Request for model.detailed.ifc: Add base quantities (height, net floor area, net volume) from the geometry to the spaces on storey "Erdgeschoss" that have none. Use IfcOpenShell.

First a look at what the model holds.

```python
import ifcopenshell
import ifcopenshell.util.element
import ifcopenshell.util.unit

model = ifcopenshell.open("model.detailed.ifc")
print(model.schema)
for unit_type in ("LENGTHUNIT", "AREAUNIT", "VOLUMEUNIT"):
    print(unit_type, ifcopenshell.util.unit.calculate_unit_scale(model, unit_type))
storey = next(s for s in model.by_type("IfcBuildingStorey") if s.Name == "Erdgeschoss")
spaces = [e for e in ifcopenshell.util.element.get_decomposition(storey) if e.is_a("IfcSpace")]
for e in sorted(spaces, key=lambda e: e.id()):
    print(e.id(), e.is_a(), e.Name, list(ifcopenshell.util.element.get_psets(e, qtos_only=True)), sep=" | ")
```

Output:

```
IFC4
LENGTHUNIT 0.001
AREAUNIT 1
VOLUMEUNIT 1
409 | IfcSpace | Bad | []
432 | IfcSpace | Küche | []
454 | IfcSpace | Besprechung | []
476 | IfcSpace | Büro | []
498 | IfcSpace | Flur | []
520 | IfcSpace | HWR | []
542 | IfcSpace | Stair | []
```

```python
import ifcopenshell
import ifcopenshell.api.pset
import ifcopenshell.geom
import ifcopenshell.util.element
import ifcopenshell.util.shape
import ifcopenshell.util.unit

model = ifcopenshell.open("model.detailed.ifc")
unit_scale = ifcopenshell.util.unit.calculate_unit_scale(model)
area_scale = ifcopenshell.util.unit.calculate_unit_scale(model, "AREAUNIT")
volume_scale = ifcopenshell.util.unit.calculate_unit_scale(model, "VOLUMEUNIT")
settings = ifcopenshell.geom.settings()

storey = next(s for s in model.by_type("IfcBuildingStorey") if s.Name == "Erdgeschoss")
spaces = [e for e in ifcopenshell.util.element.get_decomposition(storey) if e.is_a("IfcSpace")]

for e in sorted(spaces, key=lambda e: e.id()):
    if ifcopenshell.util.element.get_psets(e, qtos_only=True, should_inherit=False):
        continue
    # Geometry comes back in metres, in the element's own axes.
    shape = ifcopenshell.geom.create_shape(settings, e)
    values = {
        "Height": ifcopenshell.util.shape.get_z(shape.geometry) / unit_scale,
        "NetFloorArea": ifcopenshell.util.shape.get_footprint_area(shape.geometry) / area_scale,
        "NetVolume": ifcopenshell.util.shape.get_volume(shape.geometry) / volume_scale,
    }
    qto = ifcopenshell.api.pset.add_qto(model, product=e, name="Qto_SpaceBaseQuantities")
    ifcopenshell.api.pset.edit_qto(model, qto=qto, properties=values)
    print(e.id(), {k: round(v, 3) for k, v in values.items()})

model.write("model.detailed_edited.ifc")
```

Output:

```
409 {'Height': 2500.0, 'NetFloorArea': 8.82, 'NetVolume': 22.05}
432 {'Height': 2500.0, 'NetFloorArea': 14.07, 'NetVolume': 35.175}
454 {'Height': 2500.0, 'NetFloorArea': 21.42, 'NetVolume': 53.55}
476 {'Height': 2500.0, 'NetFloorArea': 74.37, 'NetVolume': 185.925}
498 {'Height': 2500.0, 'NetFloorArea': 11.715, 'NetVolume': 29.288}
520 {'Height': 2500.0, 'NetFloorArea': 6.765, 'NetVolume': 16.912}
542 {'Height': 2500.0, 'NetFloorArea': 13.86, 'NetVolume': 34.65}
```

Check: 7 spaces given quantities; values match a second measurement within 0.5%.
